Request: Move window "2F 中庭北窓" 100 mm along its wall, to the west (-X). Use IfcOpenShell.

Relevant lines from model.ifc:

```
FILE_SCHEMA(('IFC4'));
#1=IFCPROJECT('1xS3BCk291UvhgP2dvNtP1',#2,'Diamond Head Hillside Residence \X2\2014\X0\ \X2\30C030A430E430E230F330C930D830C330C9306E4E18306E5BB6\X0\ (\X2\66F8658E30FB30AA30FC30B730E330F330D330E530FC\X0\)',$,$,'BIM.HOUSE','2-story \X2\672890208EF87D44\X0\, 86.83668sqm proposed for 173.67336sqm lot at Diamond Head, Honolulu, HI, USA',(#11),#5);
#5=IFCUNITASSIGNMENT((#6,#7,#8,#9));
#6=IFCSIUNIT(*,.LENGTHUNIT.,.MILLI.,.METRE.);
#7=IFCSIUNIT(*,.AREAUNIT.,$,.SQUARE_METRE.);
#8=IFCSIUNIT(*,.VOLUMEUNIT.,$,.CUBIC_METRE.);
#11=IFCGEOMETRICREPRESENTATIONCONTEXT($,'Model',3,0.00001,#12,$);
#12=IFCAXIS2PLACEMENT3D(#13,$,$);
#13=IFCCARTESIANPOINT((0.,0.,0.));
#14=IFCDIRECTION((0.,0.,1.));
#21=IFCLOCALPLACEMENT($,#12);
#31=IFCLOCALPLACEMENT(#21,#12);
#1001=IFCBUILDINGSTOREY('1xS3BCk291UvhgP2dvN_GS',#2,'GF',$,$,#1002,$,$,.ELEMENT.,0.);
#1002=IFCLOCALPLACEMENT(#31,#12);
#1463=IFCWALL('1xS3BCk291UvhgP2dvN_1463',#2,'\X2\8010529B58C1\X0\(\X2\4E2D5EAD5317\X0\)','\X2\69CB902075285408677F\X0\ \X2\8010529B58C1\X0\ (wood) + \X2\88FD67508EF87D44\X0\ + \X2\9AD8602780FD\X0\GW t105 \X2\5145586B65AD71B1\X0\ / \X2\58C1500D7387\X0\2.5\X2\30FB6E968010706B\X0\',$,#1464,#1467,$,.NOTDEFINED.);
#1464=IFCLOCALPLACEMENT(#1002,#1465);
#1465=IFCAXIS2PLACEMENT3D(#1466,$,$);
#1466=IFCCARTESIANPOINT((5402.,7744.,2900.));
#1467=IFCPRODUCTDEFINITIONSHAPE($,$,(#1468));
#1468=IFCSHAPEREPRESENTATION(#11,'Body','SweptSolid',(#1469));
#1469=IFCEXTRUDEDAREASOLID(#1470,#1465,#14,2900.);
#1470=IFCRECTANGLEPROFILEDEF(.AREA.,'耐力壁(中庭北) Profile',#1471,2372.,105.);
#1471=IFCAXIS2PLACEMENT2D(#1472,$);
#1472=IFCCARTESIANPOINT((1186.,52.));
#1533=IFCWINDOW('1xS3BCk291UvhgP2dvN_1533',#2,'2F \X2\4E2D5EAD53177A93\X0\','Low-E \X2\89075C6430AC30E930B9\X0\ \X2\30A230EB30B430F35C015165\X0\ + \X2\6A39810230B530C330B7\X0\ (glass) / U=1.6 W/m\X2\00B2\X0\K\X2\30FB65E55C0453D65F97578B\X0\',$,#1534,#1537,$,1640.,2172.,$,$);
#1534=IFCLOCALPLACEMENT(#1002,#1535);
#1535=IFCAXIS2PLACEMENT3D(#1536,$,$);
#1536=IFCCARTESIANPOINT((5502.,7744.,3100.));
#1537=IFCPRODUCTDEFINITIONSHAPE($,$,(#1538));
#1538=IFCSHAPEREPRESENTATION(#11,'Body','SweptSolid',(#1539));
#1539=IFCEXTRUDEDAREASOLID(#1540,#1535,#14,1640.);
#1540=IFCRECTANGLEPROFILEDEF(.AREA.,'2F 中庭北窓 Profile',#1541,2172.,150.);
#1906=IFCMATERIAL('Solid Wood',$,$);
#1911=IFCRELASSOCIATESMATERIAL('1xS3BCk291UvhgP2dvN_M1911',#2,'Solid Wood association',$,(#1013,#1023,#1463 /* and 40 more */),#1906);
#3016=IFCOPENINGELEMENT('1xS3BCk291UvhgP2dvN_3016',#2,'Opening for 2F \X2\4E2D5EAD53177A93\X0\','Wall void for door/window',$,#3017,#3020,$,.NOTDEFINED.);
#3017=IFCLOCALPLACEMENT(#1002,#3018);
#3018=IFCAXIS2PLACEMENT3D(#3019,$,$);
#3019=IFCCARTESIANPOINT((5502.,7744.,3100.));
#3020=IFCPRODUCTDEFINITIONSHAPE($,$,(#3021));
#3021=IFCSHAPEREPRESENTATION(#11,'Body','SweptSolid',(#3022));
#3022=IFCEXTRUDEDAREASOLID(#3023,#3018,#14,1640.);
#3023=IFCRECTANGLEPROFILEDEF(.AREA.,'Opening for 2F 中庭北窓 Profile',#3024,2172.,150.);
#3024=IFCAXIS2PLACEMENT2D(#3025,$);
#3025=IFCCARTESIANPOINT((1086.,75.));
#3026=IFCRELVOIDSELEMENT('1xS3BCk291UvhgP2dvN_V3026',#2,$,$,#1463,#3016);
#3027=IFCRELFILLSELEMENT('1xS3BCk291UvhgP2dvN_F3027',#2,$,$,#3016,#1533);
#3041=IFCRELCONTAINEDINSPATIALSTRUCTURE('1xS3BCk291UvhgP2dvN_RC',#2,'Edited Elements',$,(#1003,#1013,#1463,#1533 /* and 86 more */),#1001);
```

```python
import ifcopenshell
import ifcopenshell.api.geometry
import ifcopenshell.util.placement
import ifcopenshell.util.unit

model = ifcopenshell.open("model.ifc")
unit_scale = ifcopenshell.util.unit.calculate_unit_scale(model)

window = model.by_id(1533)
opening = window.FillsVoids[0].RelatingOpeningElement
wall = opening.VoidsElements[0].RelatingBuildingElement

wall_matrix = ifcopenshell.util.placement.get_local_placement(wall.ObjectPlacement)
shift = wall_matrix[:3, 0] * -0.1 / unit_scale
before = ifcopenshell.util.placement.get_local_placement(window.ObjectPlacement)[:3, 3].copy()

# The window is not placed relative to its opening, so move both.
for product in (opening, window):
    matrix = ifcopenshell.util.placement.get_local_placement(product.ObjectPlacement)
    matrix[:3, 3] += shift
    ifcopenshell.api.geometry.edit_object_placement(model, product=product, matrix=matrix, is_si=False)

after = ifcopenshell.util.placement.get_local_placement(window.ObjectPlacement)[:3, 3]
print("window moved by", (after - before).round(3) + 0.0)

model.write("model-out.ifc")
```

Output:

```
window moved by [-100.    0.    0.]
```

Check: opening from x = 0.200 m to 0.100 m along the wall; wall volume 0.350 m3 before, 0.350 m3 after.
